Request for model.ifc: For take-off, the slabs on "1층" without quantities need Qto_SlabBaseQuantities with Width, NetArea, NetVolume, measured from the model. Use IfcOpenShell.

First a look at what the model holds.

```python
import ifcopenshell
import ifcopenshell.util.element
import ifcopenshell.util.unit

model = ifcopenshell.open("model.ifc")
print(model.schema)
for unit_type in ("LENGTHUNIT", "AREAUNIT", "VOLUMEUNIT"):
    print(unit_type, ifcopenshell.util.unit.calculate_unit_scale(model, unit_type))
storey = next(s for s in model.by_type("IfcBuildingStorey") if s.Name == "1층")
slabs = [e for e in ifcopenshell.util.element.get_decomposition(storey) if e.is_a("IfcSlab")]
for e in sorted(slabs, key=lambda e: e.id()):
    print(e.id(), e.is_a(), e.Name, list(ifcopenshell.util.element.get_psets(e, qtos_only=True)), sep=" | ")
```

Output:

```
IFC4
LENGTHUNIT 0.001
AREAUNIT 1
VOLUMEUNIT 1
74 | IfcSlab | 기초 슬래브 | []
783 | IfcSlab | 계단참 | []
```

```python
import ifcopenshell
import ifcopenshell.api.pset
import ifcopenshell.geom
import ifcopenshell.util.element
import ifcopenshell.util.shape
import ifcopenshell.util.unit

model = ifcopenshell.open("model.ifc")
unit_scale = ifcopenshell.util.unit.calculate_unit_scale(model)
area_scale = ifcopenshell.util.unit.calculate_unit_scale(model, "AREAUNIT")
volume_scale = ifcopenshell.util.unit.calculate_unit_scale(model, "VOLUMEUNIT")
settings = ifcopenshell.geom.settings()

storey = next(s for s in model.by_type("IfcBuildingStorey") if s.Name == "1층")
slabs = [e for e in ifcopenshell.util.element.get_decomposition(storey) if e.is_a("IfcSlab")]

for e in sorted(slabs, key=lambda e: e.id()):
    if ifcopenshell.util.element.get_psets(e, qtos_only=True, should_inherit=False):
        continue
    # Geometry comes back in metres, in the element's own axes.
    shape = ifcopenshell.geom.create_shape(settings, e)
    values = {
        "Width": ifcopenshell.util.shape.get_z(shape.geometry) / unit_scale,
        "NetArea": ifcopenshell.util.shape.get_footprint_area(shape.geometry) / area_scale,
        "NetVolume": ifcopenshell.util.shape.get_volume(shape.geometry) / volume_scale,
    }
    qto = ifcopenshell.api.pset.add_qto(model, product=e, name="Qto_SlabBaseQuantities")
    ifcopenshell.api.pset.edit_qto(model, qto=qto, properties=values)
    print(e.id(), {k: round(v, 3) for k, v in values.items()})

model.write("model_rev.ifc")
```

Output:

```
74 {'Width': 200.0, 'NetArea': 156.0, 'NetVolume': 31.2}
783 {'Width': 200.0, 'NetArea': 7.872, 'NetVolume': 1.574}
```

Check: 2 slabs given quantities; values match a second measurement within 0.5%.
